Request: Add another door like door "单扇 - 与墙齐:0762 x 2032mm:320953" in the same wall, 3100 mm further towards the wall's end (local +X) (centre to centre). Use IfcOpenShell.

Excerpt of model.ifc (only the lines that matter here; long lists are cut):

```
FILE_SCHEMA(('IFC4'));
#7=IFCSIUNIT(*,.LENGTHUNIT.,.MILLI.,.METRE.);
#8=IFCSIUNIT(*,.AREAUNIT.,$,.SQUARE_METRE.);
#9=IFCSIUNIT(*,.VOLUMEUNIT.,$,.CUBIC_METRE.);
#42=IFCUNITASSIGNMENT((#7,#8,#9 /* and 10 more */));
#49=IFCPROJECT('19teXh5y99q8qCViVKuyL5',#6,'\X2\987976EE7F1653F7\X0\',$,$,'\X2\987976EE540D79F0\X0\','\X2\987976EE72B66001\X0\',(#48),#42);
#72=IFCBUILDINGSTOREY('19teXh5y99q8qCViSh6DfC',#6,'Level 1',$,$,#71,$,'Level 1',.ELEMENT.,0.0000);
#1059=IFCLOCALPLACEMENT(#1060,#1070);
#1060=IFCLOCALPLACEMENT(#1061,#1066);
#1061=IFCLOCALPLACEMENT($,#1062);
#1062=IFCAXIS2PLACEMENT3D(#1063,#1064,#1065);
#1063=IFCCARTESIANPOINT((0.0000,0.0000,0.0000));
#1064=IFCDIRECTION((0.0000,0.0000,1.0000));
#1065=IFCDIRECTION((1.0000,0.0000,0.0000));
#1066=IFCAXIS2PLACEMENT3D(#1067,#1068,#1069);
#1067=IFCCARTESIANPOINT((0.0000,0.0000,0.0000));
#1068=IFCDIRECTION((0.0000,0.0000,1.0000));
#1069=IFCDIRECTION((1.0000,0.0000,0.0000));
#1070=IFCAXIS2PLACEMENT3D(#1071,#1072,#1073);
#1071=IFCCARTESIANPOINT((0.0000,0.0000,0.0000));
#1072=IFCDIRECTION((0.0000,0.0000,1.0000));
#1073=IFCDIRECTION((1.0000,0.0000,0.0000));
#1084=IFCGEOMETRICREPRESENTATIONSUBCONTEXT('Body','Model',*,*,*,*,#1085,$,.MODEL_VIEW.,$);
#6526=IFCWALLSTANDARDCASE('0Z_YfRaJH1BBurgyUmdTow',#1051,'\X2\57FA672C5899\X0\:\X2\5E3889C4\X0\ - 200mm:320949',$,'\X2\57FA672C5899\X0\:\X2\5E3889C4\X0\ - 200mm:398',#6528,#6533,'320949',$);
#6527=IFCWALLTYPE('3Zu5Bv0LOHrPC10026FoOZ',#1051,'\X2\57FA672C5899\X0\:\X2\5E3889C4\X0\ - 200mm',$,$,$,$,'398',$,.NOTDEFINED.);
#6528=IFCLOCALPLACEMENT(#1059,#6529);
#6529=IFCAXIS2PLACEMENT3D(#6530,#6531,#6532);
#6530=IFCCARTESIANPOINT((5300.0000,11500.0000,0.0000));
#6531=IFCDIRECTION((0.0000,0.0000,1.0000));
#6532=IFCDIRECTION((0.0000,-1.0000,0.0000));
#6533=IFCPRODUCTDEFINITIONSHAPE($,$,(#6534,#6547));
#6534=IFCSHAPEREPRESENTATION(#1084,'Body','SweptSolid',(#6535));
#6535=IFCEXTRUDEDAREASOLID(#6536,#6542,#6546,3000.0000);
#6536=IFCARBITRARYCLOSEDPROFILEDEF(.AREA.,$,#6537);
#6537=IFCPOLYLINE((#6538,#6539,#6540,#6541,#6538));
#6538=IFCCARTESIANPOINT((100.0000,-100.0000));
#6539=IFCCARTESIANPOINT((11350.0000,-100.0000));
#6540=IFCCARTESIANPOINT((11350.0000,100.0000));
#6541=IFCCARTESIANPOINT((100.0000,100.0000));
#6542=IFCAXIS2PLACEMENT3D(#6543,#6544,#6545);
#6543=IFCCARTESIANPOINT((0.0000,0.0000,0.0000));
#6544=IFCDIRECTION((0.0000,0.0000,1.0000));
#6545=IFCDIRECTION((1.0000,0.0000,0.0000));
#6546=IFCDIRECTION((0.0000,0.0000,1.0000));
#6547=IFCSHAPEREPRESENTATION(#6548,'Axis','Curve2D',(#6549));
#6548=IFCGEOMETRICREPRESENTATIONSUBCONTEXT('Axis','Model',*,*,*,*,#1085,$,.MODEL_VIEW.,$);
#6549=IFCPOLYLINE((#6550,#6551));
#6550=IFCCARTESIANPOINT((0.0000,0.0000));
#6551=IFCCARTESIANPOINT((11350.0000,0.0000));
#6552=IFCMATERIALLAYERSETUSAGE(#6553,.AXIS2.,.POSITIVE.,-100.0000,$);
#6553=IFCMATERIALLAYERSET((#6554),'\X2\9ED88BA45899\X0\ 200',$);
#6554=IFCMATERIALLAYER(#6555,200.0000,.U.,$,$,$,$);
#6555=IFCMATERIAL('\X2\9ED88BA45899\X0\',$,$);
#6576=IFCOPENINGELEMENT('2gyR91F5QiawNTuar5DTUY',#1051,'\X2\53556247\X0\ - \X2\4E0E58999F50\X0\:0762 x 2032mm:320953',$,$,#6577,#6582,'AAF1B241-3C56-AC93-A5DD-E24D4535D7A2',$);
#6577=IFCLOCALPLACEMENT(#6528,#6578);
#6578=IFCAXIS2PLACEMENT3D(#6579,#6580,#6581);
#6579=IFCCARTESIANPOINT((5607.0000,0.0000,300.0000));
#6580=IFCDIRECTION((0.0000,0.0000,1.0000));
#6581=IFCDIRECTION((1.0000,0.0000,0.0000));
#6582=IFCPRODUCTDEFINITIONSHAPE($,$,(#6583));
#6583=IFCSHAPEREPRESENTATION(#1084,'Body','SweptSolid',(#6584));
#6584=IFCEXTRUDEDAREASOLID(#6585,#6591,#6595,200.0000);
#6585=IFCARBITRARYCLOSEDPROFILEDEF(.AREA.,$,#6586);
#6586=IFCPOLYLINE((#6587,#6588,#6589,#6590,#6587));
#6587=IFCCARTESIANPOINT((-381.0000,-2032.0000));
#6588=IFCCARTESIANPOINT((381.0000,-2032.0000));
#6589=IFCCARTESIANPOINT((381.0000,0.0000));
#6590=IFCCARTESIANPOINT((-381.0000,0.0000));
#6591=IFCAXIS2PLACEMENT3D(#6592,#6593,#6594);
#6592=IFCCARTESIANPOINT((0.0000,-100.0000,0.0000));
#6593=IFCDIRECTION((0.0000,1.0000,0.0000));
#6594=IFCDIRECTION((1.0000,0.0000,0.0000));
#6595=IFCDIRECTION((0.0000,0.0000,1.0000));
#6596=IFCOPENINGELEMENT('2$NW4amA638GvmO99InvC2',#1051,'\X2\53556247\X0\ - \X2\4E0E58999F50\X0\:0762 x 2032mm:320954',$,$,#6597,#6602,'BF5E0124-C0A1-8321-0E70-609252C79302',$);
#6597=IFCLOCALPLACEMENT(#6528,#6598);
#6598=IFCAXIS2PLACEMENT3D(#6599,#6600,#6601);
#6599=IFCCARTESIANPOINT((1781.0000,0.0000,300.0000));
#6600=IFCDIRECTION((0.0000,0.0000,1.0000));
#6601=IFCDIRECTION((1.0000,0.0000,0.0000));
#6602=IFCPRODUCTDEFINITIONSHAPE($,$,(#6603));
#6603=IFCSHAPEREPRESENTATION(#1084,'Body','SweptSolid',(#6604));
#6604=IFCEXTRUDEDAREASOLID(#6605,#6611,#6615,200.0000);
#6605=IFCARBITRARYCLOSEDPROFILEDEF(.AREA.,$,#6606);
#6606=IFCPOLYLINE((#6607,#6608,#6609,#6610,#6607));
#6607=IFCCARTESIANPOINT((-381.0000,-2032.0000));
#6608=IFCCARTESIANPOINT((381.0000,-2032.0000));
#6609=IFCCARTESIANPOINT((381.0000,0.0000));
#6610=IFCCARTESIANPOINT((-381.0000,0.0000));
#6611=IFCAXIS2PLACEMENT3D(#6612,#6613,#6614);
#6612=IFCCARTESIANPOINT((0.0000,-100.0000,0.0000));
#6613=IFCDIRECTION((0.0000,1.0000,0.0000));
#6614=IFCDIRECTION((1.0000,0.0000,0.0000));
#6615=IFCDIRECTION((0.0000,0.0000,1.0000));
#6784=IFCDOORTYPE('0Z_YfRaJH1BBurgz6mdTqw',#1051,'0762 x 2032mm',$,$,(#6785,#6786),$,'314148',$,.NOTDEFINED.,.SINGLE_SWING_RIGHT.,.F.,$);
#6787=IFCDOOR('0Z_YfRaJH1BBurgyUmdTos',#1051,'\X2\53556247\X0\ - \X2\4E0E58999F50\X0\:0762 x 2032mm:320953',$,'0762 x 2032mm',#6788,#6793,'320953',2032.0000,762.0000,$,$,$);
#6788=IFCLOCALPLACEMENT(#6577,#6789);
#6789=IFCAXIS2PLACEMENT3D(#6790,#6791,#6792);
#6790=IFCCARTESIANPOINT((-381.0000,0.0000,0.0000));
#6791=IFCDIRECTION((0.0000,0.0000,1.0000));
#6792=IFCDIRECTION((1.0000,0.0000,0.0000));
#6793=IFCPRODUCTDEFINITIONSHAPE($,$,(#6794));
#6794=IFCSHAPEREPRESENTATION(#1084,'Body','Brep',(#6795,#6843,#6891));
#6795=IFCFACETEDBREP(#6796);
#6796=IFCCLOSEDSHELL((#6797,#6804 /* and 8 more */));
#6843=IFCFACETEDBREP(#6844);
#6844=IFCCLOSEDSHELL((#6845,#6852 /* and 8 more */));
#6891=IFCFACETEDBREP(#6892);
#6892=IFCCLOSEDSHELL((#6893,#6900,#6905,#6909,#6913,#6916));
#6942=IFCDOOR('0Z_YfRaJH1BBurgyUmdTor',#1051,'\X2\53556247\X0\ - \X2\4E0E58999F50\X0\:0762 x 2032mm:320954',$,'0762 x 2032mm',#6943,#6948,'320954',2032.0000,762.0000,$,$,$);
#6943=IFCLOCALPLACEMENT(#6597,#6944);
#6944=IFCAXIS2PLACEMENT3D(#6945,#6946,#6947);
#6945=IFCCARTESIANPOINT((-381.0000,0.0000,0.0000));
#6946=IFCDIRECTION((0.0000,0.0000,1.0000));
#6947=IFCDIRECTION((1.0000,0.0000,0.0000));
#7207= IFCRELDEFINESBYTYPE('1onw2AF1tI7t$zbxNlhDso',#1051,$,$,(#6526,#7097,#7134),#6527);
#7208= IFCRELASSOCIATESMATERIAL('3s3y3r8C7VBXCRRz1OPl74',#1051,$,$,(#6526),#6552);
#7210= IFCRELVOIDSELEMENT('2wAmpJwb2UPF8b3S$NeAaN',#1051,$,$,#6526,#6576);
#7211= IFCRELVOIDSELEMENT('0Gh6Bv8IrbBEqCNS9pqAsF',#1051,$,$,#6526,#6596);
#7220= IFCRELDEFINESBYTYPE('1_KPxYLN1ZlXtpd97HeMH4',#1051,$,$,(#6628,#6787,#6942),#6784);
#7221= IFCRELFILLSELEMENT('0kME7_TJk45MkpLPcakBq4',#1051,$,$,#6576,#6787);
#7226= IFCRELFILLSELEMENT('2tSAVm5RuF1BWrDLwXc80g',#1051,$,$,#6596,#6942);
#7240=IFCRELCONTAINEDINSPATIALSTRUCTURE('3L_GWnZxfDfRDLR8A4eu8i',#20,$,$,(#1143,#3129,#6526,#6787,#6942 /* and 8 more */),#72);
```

```python
import ifcopenshell
import ifcopenshell.api.feature
import ifcopenshell.api.geometry
import ifcopenshell.api.root
import ifcopenshell.geom
import ifcopenshell.util.element
import ifcopenshell.util.placement
import ifcopenshell.util.shape
import ifcopenshell.util.unit

model = ifcopenshell.open("model.ifc")
unit_scale = ifcopenshell.util.unit.calculate_unit_scale(model)
settings = ifcopenshell.geom.settings()


def volume(element):
    """Net volume in cubic metres, openings subtracted."""
    shape = ifcopenshell.geom.create_shape(settings, element)
    return ifcopenshell.util.shape.get_volume(shape.geometry)


def reuse_history(source, copy):
    """copy_class also copies each property set's owner history, people and application; keep the originals."""
    for rel in copy.IsDefinedBy:
        if rel.is_a("IfcRelDefinesByProperties") and (history := rel.RelatingPropertyDefinition.OwnerHistory):
            rel.RelatingPropertyDefinition.OwnerHistory = source.OwnerHistory
            ifcopenshell.util.element.remove_deep2(model, history)


door = model.by_guid("0Z_YfRaJH1BBurgyUmdTos")
opening = door.FillsVoids[0].RelatingOpeningElement
wall = opening.VoidsElements[0].RelatingBuildingElement
before = volume(wall)
shift = ifcopenshell.util.placement.get_local_placement(wall.ObjectPlacement)[:3, 0] * 3.1 / unit_scale

# copy_class copies the void relationship, type, container and properties, but no geometry.
new_opening = ifcopenshell.api.root.copy_class(model, product=opening)
new_opening.Representation = ifcopenshell.util.element.copy_deep(
    model, opening.Representation, exclude=["IfcGeometricRepresentationContext", "IfcRepresentationMap"]
)
new_opening.Name = "单扇 - 与墙齐:0762 x 2032mm"
new_opening.Tag = None
new_door = ifcopenshell.api.root.copy_class(model, product=door)
new_door.Representation = ifcopenshell.util.element.copy_deep(
    model, door.Representation, exclude=["IfcGeometricRepresentationContext", "IfcRepresentationMap"]
)
new_door.Name = "单扇 - 与墙齐:0762 x 2032mm"
new_door.Tag = None
reuse_history(door, new_door)
ifcopenshell.api.feature.add_filling(model, opening=new_opening, element=new_door)

for old, new in ((opening, new_opening), (door, new_door)):
    matrix = ifcopenshell.util.placement.get_local_placement(old.ObjectPlacement)
    matrix[:3, 3] += shift
    ifcopenshell.api.geometry.edit_object_placement(model, product=new, matrix=matrix, is_si=False)

after = volume(wall)

print(f"wall volume {before:.3f} -> {after:.3f} m3")

model.write("model_updated.ifc")
```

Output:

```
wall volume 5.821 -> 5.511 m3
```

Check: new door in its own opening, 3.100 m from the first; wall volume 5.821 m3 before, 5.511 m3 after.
